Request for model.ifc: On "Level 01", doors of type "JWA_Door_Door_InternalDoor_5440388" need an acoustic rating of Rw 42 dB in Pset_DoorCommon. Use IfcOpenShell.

First a look at what the model holds.

```python
import ifcopenshell
import ifcopenshell.util.element

model = ifcopenshell.open("model.ifc")
print(model.schema)
storey = next(s for s in model.by_type("IfcBuildingStorey") if s.Name == "Level 01")
doors = [e for e in ifcopenshell.util.element.get_decomposition(storey) if e.is_a("IfcDoor")]
seen = {}
for e in doors:
    element_type = ifcopenshell.util.element.get_type(e)
    key = (element_type.Name if element_type != e and element_type else None, ifcopenshell.util.element.get_pset(e, "Pset_DoorCommon", "AcousticRating"))
    seen[key] = seen.get(key, 0) + 1
for (name, value), count in sorted(seen.items(), key=str):
    print(count, "x", name, "|", value)
```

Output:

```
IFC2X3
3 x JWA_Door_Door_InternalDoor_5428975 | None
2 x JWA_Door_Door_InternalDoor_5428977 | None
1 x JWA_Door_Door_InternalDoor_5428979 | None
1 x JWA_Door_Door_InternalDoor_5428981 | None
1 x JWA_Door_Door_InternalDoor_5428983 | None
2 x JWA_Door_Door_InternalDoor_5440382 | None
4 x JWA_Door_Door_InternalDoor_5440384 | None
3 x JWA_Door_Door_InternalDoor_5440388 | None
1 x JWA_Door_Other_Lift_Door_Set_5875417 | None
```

```python
import ifcopenshell
import ifcopenshell.api.pset
import ifcopenshell.util.element

model = ifcopenshell.open("model.ifc")

storey = next(s for s in model.by_type("IfcBuildingStorey") if s.Name == "Level 01")
doors = [e for e in ifcopenshell.util.element.get_decomposition(storey) if e.is_a("IfcDoor")]

count = 0
for e in doors:
    element_type = ifcopenshell.util.element.get_type(e)
    if element_type in (None, e) or element_type.Name != "JWA_Door_Door_InternalDoor_5440388":
        continue
    # add_pset returns the element's existing set when there is one.
    pset = ifcopenshell.api.pset.add_pset(model, product=e, name="Pset_DoorCommon")
    ifcopenshell.api.pset.edit_pset(model, pset=pset, properties={"AcousticRating": "Rw 42 dB"})
    count += 1

print(count, "doors updated")

model.write("model_v2.ifc")
```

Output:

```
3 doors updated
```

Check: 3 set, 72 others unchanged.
